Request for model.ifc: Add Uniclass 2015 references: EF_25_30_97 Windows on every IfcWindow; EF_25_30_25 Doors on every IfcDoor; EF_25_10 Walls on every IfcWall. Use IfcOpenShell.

First a look at what the model holds.

```python
import ifcopenshell

model = ifcopenshell.open("model.ifc")
print(model.schema)
print("classifications:", [c.Name for c in model.by_type("IfcClassification")])
for ifc_class in ("IfcDoor", "IfcRoof", "IfcStair", "IfcWall", "IfcWindow"):
    print(ifc_class, len(model.by_type(ifc_class)))
```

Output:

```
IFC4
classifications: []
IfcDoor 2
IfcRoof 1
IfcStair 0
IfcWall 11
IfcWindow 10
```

```python
import ifcopenshell
import ifcopenshell.api.classification

model = ifcopenshell.open("model.ifc")

system = ifcopenshell.api.classification.add_classification(model, classification="Uniclass 2015")

codes = {
    "IfcWindow": ("EF_25_30_97", "Windows"),
    "IfcDoor": ("EF_25_30_25", "Doors"),
    "IfcWall": ("EF_25_10", "Walls"),
}
for ifc_class, (code, name) in codes.items():
    products = model.by_type(ifc_class)
    ifcopenshell.api.classification.add_reference(
        model, products=products, classification=system, identification=code, name=name
    )
    print(code, len(products))

model.write("model_edited.ifc")
```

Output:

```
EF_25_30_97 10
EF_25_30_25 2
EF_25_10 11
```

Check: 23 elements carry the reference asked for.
